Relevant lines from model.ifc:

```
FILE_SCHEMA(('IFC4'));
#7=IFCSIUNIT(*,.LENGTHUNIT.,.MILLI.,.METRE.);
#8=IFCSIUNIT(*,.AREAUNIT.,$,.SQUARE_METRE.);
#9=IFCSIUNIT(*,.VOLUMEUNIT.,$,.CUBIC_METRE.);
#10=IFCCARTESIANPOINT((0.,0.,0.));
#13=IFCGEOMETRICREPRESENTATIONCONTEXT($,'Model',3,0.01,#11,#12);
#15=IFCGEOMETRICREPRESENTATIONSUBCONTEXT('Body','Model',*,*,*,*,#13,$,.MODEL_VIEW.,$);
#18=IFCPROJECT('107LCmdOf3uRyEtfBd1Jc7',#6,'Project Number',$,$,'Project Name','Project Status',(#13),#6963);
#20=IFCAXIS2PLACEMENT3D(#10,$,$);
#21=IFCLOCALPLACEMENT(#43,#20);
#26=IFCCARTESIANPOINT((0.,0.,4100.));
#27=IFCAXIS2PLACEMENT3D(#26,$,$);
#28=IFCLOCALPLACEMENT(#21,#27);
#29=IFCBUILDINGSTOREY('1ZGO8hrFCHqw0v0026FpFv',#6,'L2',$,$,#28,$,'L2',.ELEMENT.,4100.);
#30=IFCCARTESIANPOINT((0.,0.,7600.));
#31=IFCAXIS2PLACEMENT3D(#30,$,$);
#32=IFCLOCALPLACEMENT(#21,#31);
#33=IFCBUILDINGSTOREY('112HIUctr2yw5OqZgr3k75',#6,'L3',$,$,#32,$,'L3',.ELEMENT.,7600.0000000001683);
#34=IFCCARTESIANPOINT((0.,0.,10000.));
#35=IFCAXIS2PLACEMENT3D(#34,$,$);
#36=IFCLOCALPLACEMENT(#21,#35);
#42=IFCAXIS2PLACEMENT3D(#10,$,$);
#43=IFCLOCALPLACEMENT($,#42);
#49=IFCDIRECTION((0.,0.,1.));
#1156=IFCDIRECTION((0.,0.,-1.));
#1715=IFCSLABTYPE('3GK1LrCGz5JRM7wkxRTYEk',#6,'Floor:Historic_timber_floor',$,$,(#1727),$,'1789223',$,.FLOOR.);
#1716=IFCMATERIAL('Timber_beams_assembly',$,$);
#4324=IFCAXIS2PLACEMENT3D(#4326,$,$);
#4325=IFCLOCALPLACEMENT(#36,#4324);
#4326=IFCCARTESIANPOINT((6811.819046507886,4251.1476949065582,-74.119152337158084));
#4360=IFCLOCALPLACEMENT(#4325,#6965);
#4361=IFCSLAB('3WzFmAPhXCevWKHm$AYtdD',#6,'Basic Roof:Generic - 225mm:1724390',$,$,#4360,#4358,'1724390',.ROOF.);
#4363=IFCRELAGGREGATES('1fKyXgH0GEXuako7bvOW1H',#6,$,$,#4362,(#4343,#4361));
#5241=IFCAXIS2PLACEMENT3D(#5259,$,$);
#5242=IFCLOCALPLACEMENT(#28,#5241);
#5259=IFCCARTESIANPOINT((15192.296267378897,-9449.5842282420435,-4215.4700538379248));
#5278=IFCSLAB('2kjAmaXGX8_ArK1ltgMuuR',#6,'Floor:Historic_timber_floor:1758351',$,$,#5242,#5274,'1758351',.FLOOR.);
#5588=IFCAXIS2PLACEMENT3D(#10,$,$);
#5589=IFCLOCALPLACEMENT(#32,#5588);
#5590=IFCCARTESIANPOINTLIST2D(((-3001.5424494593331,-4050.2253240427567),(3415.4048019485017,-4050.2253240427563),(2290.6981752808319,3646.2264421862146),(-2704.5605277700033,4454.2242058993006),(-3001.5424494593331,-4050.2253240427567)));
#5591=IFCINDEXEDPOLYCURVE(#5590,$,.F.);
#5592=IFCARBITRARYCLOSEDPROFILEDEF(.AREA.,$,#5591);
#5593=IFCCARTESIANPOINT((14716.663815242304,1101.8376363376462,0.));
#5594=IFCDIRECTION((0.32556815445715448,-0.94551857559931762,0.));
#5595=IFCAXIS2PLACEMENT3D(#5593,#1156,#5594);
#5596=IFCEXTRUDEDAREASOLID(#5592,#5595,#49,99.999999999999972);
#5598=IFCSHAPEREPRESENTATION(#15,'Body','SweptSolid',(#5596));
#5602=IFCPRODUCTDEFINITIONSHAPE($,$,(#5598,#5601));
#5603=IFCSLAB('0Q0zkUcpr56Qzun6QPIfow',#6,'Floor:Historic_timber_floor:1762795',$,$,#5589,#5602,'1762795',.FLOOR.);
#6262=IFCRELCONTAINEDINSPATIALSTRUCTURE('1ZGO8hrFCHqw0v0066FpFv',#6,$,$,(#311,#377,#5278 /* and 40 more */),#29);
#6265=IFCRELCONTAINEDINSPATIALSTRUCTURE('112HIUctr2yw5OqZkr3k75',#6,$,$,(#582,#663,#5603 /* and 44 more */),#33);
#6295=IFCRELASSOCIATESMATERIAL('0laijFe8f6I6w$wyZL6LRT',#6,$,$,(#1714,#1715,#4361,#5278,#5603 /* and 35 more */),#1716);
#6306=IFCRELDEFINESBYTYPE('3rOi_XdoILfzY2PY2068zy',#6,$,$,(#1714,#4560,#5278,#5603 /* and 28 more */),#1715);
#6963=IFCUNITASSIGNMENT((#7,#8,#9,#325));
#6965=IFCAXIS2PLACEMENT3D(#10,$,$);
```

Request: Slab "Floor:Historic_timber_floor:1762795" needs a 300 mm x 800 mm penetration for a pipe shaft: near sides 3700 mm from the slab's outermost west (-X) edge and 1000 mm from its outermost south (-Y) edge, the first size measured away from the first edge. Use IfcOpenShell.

```python
import numpy as np
import ifcopenshell
import ifcopenshell.api.feature
import ifcopenshell.api.geometry
import ifcopenshell.api.root
import ifcopenshell.geom
import ifcopenshell.util.placement
import ifcopenshell.util.representation
import ifcopenshell.util.shape
import ifcopenshell.util.unit

model = ifcopenshell.open("model.ifc")
unit_scale = ifcopenshell.util.unit.calculate_unit_scale(model)
settings = ifcopenshell.geom.settings()


def volume(element):
    """Net volume in cubic metres, openings subtracted."""
    shape = ifcopenshell.geom.create_shape(settings, element)
    return ifcopenshell.util.shape.get_volume(shape.geometry)


slab = model.by_guid("0Q0zkUcpr56Qzun6QPIfow")
before = volume(slab)

# Extent in the slab's own axes, in metres. The edges named are its -X and -Y sides.
slab_shape = ifcopenshell.geom.create_shape(settings, slab)
vertices = ifcopenshell.util.shape.get_vertices(slab_shape.geometry)
x_min, y_min, bottom = vertices.min(axis=0)
top = vertices[:, 2].max()

opening = ifcopenshell.api.root.create_entity(model, ifc_class="IfcOpeningElement", name="Pipe shaft opening", predefined_type="OPENING")
context = ifcopenshell.util.representation.get_context(model, "Model", "Body", "MODEL_VIEW")
width, depth = 0.3, 0.8
outline = [(0.0, 0.0), (width, 0.0), (width, depth), (0.0, depth), (0.0, 0.0)]
# Overshoot both faces by 50 mm so the cut is clean.
shape = ifcopenshell.api.geometry.add_slab_representation(
    model, context=context, depth=top - bottom + 0.1, polyline=outline
)
ifcopenshell.api.geometry.assign_representation(model, product=opening, representation=shape)

matrix = ifcopenshell.util.placement.get_local_placement(slab.ObjectPlacement)
matrix[:, 3] = matrix @ np.append(np.array([x_min + 3.7, y_min + 1, bottom - 0.05]) / unit_scale, 1.0)
ifcopenshell.api.geometry.edit_object_placement(model, product=opening, matrix=matrix, is_si=False)
ifcopenshell.api.feature.add_feature(model, feature=opening, element=slab)

after = volume(slab)

print(f"slab volume {before:.3f} -> {after:.3f} m3")

model.write("model_rev.ifc")
```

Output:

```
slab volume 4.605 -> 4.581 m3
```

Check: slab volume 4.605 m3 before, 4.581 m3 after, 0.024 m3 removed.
